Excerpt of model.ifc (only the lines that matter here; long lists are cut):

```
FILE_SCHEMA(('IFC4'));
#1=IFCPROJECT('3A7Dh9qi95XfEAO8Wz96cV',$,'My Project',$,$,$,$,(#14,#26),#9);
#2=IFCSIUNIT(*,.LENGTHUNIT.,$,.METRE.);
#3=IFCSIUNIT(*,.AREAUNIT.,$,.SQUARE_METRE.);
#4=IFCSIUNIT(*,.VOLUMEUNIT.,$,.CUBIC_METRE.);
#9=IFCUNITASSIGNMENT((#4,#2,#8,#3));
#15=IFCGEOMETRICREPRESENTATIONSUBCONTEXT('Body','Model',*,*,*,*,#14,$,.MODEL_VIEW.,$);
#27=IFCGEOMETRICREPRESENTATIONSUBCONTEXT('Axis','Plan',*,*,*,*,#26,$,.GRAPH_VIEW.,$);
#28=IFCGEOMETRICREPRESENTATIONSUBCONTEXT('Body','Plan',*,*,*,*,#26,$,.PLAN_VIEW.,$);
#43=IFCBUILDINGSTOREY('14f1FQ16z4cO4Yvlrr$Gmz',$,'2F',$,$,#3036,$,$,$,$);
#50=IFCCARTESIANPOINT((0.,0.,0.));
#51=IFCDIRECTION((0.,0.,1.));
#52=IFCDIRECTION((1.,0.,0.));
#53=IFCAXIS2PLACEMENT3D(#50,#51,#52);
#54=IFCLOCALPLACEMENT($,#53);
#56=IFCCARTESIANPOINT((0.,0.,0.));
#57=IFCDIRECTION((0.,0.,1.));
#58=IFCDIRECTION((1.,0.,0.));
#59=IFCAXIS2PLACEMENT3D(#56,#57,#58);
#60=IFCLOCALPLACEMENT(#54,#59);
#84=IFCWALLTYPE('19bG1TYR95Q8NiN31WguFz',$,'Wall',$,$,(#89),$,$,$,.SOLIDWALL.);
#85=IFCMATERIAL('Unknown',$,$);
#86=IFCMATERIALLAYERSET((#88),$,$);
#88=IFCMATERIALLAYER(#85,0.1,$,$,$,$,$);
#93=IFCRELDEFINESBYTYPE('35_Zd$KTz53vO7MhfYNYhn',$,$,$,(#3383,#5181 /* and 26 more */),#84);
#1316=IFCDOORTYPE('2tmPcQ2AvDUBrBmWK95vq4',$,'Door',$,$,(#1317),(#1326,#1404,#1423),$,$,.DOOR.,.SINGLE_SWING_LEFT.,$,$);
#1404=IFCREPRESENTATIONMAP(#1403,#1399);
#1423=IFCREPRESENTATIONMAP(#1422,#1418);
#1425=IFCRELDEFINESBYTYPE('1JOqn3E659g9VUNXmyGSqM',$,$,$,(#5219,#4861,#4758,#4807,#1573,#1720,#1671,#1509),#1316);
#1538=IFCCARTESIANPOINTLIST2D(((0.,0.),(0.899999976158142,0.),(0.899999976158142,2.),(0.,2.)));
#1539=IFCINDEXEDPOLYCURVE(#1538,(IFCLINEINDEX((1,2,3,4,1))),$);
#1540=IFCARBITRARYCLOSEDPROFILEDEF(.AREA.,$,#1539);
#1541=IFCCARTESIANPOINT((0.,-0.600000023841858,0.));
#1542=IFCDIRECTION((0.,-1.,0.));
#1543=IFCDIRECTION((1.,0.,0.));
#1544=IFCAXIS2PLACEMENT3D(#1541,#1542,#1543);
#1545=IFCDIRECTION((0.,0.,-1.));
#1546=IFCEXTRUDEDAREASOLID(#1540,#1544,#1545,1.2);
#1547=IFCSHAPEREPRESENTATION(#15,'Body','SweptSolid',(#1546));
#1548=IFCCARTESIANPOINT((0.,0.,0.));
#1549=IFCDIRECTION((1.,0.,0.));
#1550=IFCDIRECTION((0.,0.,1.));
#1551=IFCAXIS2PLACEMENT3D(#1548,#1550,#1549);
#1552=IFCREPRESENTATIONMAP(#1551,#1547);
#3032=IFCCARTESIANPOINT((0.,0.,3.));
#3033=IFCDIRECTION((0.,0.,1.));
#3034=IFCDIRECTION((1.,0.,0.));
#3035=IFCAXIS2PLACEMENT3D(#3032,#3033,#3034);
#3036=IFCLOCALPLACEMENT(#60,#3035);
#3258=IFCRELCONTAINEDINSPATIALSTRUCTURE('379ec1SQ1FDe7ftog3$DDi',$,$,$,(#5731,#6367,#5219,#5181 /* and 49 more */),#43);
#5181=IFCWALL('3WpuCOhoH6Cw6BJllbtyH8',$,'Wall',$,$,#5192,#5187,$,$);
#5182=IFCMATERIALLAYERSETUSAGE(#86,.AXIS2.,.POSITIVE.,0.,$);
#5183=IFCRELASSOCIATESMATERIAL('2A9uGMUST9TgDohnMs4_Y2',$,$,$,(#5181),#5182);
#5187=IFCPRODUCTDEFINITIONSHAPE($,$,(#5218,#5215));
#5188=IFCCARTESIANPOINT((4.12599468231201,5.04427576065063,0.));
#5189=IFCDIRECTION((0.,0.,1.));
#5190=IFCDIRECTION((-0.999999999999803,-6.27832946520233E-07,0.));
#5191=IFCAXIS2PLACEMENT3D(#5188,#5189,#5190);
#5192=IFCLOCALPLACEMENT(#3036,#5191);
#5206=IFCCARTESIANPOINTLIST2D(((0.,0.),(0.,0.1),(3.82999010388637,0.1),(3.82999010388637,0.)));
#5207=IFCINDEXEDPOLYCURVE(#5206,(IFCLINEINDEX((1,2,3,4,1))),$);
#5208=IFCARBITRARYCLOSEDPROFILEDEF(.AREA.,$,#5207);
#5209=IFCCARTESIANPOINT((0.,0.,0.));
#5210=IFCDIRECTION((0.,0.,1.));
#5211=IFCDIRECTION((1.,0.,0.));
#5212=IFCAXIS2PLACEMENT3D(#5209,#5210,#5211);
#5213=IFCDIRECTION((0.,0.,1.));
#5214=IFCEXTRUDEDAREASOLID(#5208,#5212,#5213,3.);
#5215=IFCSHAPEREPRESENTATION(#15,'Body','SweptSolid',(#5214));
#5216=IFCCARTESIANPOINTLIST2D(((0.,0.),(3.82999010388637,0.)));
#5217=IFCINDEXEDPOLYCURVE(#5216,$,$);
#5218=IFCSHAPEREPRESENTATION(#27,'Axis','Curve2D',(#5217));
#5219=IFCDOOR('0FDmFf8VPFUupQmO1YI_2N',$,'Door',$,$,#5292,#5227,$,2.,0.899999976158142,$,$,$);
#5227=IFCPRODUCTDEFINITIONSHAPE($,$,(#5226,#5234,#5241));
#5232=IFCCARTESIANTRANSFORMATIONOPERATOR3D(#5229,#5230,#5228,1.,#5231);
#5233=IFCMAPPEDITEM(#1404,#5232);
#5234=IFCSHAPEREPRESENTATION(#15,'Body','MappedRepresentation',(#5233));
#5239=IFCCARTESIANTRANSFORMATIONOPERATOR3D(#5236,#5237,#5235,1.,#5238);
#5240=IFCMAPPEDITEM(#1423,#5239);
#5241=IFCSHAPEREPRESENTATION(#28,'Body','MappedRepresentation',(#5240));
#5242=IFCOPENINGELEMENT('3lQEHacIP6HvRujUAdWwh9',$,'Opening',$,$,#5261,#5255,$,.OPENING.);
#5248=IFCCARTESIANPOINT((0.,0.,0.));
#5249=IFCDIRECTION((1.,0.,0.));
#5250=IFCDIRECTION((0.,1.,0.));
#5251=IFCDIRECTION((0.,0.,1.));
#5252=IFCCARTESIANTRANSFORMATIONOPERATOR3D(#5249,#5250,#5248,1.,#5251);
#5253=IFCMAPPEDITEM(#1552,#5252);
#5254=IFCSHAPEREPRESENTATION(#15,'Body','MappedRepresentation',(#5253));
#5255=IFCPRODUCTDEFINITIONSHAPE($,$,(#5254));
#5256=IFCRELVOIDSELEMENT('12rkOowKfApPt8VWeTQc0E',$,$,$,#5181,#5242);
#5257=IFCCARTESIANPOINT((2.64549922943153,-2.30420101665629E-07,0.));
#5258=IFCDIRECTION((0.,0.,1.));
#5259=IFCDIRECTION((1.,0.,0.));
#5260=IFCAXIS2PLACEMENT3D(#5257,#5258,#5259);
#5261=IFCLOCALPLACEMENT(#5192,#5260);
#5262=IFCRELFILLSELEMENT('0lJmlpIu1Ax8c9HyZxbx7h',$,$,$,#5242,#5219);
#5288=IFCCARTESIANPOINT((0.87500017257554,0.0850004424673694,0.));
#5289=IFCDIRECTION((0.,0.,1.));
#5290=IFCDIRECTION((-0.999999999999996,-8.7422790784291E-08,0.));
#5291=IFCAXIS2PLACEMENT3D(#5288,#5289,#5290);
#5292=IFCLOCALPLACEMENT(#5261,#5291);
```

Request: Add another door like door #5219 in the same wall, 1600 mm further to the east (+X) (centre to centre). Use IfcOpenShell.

```python
import ifcopenshell
import ifcopenshell.api.feature
import ifcopenshell.api.geometry
import ifcopenshell.api.root
import ifcopenshell.geom
import ifcopenshell.util.element
import ifcopenshell.util.placement
import ifcopenshell.util.shape
import ifcopenshell.util.unit

model = ifcopenshell.open("model.ifc")
unit_scale = ifcopenshell.util.unit.calculate_unit_scale(model)
settings = ifcopenshell.geom.settings()


def volume(element):
    """Net volume in cubic metres, openings subtracted."""
    shape = ifcopenshell.geom.create_shape(settings, element)
    return ifcopenshell.util.shape.get_volume(shape.geometry)


door = model.by_id(5219)
opening = door.FillsVoids[0].RelatingOpeningElement
wall = opening.VoidsElements[0].RelatingBuildingElement
before = volume(wall)
shift = ifcopenshell.util.placement.get_local_placement(wall.ObjectPlacement)[:3, 0] * -1.6 / unit_scale

# copy_class copies the void relationship, type, container and properties, but no geometry.
new_opening = ifcopenshell.api.root.copy_class(model, product=opening)
new_opening.Representation = ifcopenshell.util.element.copy_deep(
    model, opening.Representation, exclude=["IfcGeometricRepresentationContext", "IfcRepresentationMap"]
)
new_door = ifcopenshell.api.root.copy_class(model, product=door)
new_door.Representation = ifcopenshell.util.element.copy_deep(
    model, door.Representation, exclude=["IfcGeometricRepresentationContext", "IfcRepresentationMap"]
)
ifcopenshell.api.feature.add_filling(model, opening=new_opening, element=new_door)

for old, new in ((opening, new_opening), (door, new_door)):
    matrix = ifcopenshell.util.placement.get_local_placement(old.ObjectPlacement)
    matrix[:3, 3] += shift
    ifcopenshell.api.geometry.edit_object_placement(model, product=new, matrix=matrix, is_si=False)

after = volume(wall)

print(f"wall volume {before:.3f} -> {after:.3f} m3")

model.write("model_updated.ifc")
```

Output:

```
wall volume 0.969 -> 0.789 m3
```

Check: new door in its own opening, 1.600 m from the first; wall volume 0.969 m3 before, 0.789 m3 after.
